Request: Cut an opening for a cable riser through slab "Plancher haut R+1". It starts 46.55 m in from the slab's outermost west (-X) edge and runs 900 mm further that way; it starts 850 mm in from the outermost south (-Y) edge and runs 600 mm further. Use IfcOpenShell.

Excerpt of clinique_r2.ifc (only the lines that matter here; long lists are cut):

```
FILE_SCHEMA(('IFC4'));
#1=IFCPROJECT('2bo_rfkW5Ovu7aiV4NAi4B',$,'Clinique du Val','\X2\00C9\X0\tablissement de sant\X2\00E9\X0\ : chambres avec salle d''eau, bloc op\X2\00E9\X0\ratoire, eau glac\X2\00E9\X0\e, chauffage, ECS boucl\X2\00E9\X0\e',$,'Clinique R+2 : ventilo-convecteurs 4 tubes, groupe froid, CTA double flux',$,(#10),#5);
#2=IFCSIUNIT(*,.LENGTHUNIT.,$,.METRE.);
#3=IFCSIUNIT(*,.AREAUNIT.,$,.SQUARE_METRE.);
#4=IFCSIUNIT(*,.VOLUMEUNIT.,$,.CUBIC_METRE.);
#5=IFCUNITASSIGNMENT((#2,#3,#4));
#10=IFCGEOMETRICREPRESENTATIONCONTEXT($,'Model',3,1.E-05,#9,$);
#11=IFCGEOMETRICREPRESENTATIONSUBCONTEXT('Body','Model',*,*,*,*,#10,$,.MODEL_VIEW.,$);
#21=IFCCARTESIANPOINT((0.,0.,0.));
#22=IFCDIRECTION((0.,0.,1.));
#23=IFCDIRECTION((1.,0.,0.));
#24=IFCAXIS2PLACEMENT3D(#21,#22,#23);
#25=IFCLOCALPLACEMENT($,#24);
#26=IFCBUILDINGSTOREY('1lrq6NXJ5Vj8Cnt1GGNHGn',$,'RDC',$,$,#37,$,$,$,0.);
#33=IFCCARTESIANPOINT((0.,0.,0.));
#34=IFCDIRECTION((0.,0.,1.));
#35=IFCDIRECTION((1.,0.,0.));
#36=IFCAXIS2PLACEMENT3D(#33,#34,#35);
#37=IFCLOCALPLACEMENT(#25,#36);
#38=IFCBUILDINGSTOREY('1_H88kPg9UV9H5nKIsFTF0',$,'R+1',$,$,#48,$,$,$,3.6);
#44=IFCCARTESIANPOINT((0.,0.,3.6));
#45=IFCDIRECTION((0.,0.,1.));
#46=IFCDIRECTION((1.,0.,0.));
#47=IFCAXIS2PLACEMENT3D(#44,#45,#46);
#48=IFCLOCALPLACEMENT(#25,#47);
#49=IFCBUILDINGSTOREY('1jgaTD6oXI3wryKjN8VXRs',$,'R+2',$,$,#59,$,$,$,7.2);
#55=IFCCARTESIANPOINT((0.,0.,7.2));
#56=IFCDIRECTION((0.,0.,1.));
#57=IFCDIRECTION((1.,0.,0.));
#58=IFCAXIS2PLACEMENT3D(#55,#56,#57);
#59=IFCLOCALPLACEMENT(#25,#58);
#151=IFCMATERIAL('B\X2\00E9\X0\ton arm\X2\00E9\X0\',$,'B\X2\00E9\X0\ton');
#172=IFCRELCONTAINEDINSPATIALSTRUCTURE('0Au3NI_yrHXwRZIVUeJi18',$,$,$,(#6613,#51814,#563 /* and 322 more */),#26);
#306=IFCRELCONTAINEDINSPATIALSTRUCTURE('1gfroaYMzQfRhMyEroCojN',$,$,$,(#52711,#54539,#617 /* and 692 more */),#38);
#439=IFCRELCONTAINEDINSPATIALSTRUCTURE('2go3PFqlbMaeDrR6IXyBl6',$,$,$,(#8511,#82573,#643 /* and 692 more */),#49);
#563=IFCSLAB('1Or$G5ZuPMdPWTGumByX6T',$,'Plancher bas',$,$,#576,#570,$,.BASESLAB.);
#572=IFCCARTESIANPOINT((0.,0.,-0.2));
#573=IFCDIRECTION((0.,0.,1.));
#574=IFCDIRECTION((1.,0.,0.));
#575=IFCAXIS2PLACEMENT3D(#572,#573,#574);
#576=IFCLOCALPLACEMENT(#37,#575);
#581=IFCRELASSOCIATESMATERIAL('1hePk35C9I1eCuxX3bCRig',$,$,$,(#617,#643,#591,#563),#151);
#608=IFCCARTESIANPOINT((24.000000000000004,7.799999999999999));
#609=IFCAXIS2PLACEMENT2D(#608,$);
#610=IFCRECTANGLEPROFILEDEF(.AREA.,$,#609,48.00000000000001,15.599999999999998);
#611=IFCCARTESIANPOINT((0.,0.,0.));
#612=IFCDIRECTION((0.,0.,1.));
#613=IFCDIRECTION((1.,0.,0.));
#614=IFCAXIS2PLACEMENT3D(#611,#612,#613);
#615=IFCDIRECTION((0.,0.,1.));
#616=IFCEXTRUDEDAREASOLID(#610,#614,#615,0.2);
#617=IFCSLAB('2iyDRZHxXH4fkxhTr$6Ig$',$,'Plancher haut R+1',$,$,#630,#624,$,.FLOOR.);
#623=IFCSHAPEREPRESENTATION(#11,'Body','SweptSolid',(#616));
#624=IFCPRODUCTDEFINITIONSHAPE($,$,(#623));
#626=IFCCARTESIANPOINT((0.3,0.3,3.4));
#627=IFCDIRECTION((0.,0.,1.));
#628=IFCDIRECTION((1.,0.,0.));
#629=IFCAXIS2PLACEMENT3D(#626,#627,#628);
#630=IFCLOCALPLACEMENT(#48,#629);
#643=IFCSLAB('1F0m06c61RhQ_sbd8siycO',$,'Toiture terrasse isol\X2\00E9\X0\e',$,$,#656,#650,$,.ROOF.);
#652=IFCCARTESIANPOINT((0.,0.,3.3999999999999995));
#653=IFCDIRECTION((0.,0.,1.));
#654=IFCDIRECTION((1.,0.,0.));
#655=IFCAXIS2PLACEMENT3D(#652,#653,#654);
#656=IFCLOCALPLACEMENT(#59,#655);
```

```python
import numpy as np
import ifcopenshell
import ifcopenshell.api.feature
import ifcopenshell.api.geometry
import ifcopenshell.api.root
import ifcopenshell.geom
import ifcopenshell.util.placement
import ifcopenshell.util.representation
import ifcopenshell.util.shape
import ifcopenshell.util.unit

model = ifcopenshell.open("clinique_r2.ifc")
unit_scale = ifcopenshell.util.unit.calculate_unit_scale(model)
settings = ifcopenshell.geom.settings()


def volume(element):
    """Net volume in cubic metres, openings subtracted."""
    shape = ifcopenshell.geom.create_shape(settings, element)
    return ifcopenshell.util.shape.get_volume(shape.geometry)


slab = model.by_guid("2iyDRZHxXH4fkxhTr$6Ig$")
before = volume(slab)

# Extent in the slab's own axes, in metres. The edges named are its -X and -Y sides.
slab_shape = ifcopenshell.geom.create_shape(settings, slab)
vertices = ifcopenshell.util.shape.get_vertices(slab_shape.geometry)
x_min, y_min, bottom = vertices.min(axis=0)
top = vertices[:, 2].max()

opening = ifcopenshell.api.root.create_entity(model, ifc_class="IfcOpeningElement", name="Cable riser opening", predefined_type="OPENING")
context = ifcopenshell.util.representation.get_context(model, "Model", "Body", "MODEL_VIEW")
width, depth = 0.9, 0.6
outline = [(0.0, 0.0), (width, 0.0), (width, depth), (0.0, depth), (0.0, 0.0)]
# Overshoot both faces by 50 mm so the cut is clean.
shape = ifcopenshell.api.geometry.add_slab_representation(
    model, context=context, depth=top - bottom + 0.1, polyline=outline
)
ifcopenshell.api.geometry.assign_representation(model, product=opening, representation=shape)

matrix = ifcopenshell.util.placement.get_local_placement(slab.ObjectPlacement)
matrix[:, 3] = matrix @ np.append(np.array([x_min + 46.55, y_min + 0.85, bottom - 0.05]) / unit_scale, 1.0)
ifcopenshell.api.geometry.edit_object_placement(model, product=opening, matrix=matrix, is_si=False)
ifcopenshell.api.feature.add_feature(model, feature=opening, element=slab)

after = volume(slab)

print(f"slab volume {before:.3f} -> {after:.3f} m3")

model.write("clinique_r2-out.ifc")
```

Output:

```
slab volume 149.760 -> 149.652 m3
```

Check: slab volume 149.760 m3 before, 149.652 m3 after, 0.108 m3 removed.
